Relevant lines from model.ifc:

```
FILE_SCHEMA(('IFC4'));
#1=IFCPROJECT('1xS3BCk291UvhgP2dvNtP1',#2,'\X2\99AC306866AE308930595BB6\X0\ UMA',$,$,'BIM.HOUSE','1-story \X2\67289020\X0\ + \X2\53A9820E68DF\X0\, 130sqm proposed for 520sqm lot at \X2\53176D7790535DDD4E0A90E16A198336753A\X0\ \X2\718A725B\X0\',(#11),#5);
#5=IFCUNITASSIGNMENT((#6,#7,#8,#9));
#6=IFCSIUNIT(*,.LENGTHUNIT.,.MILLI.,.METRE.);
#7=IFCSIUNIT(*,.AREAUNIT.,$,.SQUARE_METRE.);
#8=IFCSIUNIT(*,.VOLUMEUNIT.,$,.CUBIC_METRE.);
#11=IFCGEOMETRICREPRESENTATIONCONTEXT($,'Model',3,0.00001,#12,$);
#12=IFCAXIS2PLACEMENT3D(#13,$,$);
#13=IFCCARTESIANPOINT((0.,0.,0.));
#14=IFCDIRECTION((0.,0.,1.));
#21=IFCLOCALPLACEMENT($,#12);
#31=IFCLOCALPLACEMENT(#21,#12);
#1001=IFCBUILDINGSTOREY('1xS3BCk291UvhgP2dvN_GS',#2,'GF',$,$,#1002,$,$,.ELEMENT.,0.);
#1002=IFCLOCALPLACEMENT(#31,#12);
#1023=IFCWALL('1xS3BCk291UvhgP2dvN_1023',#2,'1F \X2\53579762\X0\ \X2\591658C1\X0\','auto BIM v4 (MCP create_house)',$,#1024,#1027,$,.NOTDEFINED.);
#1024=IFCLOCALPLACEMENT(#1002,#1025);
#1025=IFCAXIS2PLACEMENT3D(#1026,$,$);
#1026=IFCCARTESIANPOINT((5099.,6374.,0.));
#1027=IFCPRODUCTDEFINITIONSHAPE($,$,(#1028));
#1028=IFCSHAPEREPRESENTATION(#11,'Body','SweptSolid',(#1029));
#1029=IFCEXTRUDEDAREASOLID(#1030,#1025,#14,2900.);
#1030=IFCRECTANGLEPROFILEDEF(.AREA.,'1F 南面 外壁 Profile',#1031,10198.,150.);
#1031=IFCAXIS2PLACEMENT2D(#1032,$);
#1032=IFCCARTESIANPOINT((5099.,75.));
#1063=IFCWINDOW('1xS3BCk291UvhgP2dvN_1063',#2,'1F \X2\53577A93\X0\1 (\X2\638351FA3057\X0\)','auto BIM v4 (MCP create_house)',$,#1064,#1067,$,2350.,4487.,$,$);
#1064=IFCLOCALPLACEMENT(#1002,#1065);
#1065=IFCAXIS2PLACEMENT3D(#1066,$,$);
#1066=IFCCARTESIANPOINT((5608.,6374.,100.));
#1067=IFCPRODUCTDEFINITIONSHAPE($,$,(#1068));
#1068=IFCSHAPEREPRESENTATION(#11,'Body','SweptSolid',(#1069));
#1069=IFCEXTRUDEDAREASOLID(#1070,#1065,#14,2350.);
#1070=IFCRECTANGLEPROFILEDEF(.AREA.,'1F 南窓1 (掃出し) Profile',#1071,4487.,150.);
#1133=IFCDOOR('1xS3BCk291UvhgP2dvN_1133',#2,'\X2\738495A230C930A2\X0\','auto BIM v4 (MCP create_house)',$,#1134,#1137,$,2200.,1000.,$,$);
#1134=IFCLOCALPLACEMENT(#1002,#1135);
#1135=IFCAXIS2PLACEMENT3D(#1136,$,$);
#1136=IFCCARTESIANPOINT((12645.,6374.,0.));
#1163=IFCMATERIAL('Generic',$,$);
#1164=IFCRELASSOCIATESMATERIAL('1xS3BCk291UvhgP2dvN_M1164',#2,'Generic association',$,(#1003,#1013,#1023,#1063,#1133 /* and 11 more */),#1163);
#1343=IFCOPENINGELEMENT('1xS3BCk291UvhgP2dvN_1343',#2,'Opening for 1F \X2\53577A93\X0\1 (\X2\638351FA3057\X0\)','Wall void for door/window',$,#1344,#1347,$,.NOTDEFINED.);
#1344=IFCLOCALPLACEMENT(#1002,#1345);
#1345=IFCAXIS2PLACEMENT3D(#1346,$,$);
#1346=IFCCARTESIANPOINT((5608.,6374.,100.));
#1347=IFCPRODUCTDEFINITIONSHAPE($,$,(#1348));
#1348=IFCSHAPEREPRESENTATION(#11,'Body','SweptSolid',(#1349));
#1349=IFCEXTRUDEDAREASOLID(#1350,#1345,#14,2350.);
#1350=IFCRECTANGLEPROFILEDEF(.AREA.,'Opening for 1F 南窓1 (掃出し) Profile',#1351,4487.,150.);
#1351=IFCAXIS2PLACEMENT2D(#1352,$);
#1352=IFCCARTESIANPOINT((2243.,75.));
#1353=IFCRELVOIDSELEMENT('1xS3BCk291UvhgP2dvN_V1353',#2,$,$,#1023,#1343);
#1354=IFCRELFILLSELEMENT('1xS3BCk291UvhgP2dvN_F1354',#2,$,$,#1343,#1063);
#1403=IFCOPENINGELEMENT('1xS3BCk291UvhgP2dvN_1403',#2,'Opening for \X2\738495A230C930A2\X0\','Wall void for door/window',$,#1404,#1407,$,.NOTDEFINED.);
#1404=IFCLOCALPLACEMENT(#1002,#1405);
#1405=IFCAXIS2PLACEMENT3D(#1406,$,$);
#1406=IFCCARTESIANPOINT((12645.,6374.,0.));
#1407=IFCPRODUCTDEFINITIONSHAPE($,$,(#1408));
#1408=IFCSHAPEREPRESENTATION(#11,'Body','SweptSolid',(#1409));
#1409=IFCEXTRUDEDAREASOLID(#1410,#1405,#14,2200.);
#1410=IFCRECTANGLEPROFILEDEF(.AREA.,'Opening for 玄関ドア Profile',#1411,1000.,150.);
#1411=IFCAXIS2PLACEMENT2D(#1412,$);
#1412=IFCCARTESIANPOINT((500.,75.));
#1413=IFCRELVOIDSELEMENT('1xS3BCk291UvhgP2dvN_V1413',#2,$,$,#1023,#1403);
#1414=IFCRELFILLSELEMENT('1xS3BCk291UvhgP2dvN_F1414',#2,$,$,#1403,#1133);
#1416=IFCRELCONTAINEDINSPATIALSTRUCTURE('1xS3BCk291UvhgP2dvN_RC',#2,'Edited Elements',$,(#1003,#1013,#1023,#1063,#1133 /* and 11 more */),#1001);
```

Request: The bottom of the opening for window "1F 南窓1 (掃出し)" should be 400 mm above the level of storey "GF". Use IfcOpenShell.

```python
import numpy as np
import ifcopenshell
import ifcopenshell.api.geometry
import ifcopenshell.geom
import ifcopenshell.util.element
import ifcopenshell.util.placement
import ifcopenshell.util.shape
import ifcopenshell.util.unit

model = ifcopenshell.open("model.ifc")
unit_scale = ifcopenshell.util.unit.calculate_unit_scale(model)

window = model.by_guid("1xS3BCk291UvhgP2dvN_1063")
opening = window.FillsVoids[0].RelatingOpeningElement
storey = ifcopenshell.util.element.get_container(window, ifc_class="IfcBuildingStorey")
level = ifcopenshell.util.placement.get_local_placement(storey.ObjectPlacement)[2, 3]

# The opening's origin need not be at the sill, so measure its lowest point.
shape = ifcopenshell.geom.create_shape(ifcopenshell.geom.settings(), opening)
bottom = ifcopenshell.util.shape.get_shape_bottom_elevation(shape, shape.geometry) / unit_scale
dz = level + 400.0 - bottom

shift = np.array([0.0, 0.0, dz])
# The window is not placed relative to its opening, so move both.
for product in (opening, window):
    matrix = ifcopenshell.util.placement.get_local_placement(product.ObjectPlacement)
    matrix[:3, 3] += shift
    ifcopenshell.api.geometry.edit_object_placement(model, product=product, matrix=matrix, is_si=False)

print(f"moved by {dz * unit_scale:+.3f} m")

model.write("model-out.ifc")
```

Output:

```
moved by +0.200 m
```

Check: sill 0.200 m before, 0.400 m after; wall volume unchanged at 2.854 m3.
